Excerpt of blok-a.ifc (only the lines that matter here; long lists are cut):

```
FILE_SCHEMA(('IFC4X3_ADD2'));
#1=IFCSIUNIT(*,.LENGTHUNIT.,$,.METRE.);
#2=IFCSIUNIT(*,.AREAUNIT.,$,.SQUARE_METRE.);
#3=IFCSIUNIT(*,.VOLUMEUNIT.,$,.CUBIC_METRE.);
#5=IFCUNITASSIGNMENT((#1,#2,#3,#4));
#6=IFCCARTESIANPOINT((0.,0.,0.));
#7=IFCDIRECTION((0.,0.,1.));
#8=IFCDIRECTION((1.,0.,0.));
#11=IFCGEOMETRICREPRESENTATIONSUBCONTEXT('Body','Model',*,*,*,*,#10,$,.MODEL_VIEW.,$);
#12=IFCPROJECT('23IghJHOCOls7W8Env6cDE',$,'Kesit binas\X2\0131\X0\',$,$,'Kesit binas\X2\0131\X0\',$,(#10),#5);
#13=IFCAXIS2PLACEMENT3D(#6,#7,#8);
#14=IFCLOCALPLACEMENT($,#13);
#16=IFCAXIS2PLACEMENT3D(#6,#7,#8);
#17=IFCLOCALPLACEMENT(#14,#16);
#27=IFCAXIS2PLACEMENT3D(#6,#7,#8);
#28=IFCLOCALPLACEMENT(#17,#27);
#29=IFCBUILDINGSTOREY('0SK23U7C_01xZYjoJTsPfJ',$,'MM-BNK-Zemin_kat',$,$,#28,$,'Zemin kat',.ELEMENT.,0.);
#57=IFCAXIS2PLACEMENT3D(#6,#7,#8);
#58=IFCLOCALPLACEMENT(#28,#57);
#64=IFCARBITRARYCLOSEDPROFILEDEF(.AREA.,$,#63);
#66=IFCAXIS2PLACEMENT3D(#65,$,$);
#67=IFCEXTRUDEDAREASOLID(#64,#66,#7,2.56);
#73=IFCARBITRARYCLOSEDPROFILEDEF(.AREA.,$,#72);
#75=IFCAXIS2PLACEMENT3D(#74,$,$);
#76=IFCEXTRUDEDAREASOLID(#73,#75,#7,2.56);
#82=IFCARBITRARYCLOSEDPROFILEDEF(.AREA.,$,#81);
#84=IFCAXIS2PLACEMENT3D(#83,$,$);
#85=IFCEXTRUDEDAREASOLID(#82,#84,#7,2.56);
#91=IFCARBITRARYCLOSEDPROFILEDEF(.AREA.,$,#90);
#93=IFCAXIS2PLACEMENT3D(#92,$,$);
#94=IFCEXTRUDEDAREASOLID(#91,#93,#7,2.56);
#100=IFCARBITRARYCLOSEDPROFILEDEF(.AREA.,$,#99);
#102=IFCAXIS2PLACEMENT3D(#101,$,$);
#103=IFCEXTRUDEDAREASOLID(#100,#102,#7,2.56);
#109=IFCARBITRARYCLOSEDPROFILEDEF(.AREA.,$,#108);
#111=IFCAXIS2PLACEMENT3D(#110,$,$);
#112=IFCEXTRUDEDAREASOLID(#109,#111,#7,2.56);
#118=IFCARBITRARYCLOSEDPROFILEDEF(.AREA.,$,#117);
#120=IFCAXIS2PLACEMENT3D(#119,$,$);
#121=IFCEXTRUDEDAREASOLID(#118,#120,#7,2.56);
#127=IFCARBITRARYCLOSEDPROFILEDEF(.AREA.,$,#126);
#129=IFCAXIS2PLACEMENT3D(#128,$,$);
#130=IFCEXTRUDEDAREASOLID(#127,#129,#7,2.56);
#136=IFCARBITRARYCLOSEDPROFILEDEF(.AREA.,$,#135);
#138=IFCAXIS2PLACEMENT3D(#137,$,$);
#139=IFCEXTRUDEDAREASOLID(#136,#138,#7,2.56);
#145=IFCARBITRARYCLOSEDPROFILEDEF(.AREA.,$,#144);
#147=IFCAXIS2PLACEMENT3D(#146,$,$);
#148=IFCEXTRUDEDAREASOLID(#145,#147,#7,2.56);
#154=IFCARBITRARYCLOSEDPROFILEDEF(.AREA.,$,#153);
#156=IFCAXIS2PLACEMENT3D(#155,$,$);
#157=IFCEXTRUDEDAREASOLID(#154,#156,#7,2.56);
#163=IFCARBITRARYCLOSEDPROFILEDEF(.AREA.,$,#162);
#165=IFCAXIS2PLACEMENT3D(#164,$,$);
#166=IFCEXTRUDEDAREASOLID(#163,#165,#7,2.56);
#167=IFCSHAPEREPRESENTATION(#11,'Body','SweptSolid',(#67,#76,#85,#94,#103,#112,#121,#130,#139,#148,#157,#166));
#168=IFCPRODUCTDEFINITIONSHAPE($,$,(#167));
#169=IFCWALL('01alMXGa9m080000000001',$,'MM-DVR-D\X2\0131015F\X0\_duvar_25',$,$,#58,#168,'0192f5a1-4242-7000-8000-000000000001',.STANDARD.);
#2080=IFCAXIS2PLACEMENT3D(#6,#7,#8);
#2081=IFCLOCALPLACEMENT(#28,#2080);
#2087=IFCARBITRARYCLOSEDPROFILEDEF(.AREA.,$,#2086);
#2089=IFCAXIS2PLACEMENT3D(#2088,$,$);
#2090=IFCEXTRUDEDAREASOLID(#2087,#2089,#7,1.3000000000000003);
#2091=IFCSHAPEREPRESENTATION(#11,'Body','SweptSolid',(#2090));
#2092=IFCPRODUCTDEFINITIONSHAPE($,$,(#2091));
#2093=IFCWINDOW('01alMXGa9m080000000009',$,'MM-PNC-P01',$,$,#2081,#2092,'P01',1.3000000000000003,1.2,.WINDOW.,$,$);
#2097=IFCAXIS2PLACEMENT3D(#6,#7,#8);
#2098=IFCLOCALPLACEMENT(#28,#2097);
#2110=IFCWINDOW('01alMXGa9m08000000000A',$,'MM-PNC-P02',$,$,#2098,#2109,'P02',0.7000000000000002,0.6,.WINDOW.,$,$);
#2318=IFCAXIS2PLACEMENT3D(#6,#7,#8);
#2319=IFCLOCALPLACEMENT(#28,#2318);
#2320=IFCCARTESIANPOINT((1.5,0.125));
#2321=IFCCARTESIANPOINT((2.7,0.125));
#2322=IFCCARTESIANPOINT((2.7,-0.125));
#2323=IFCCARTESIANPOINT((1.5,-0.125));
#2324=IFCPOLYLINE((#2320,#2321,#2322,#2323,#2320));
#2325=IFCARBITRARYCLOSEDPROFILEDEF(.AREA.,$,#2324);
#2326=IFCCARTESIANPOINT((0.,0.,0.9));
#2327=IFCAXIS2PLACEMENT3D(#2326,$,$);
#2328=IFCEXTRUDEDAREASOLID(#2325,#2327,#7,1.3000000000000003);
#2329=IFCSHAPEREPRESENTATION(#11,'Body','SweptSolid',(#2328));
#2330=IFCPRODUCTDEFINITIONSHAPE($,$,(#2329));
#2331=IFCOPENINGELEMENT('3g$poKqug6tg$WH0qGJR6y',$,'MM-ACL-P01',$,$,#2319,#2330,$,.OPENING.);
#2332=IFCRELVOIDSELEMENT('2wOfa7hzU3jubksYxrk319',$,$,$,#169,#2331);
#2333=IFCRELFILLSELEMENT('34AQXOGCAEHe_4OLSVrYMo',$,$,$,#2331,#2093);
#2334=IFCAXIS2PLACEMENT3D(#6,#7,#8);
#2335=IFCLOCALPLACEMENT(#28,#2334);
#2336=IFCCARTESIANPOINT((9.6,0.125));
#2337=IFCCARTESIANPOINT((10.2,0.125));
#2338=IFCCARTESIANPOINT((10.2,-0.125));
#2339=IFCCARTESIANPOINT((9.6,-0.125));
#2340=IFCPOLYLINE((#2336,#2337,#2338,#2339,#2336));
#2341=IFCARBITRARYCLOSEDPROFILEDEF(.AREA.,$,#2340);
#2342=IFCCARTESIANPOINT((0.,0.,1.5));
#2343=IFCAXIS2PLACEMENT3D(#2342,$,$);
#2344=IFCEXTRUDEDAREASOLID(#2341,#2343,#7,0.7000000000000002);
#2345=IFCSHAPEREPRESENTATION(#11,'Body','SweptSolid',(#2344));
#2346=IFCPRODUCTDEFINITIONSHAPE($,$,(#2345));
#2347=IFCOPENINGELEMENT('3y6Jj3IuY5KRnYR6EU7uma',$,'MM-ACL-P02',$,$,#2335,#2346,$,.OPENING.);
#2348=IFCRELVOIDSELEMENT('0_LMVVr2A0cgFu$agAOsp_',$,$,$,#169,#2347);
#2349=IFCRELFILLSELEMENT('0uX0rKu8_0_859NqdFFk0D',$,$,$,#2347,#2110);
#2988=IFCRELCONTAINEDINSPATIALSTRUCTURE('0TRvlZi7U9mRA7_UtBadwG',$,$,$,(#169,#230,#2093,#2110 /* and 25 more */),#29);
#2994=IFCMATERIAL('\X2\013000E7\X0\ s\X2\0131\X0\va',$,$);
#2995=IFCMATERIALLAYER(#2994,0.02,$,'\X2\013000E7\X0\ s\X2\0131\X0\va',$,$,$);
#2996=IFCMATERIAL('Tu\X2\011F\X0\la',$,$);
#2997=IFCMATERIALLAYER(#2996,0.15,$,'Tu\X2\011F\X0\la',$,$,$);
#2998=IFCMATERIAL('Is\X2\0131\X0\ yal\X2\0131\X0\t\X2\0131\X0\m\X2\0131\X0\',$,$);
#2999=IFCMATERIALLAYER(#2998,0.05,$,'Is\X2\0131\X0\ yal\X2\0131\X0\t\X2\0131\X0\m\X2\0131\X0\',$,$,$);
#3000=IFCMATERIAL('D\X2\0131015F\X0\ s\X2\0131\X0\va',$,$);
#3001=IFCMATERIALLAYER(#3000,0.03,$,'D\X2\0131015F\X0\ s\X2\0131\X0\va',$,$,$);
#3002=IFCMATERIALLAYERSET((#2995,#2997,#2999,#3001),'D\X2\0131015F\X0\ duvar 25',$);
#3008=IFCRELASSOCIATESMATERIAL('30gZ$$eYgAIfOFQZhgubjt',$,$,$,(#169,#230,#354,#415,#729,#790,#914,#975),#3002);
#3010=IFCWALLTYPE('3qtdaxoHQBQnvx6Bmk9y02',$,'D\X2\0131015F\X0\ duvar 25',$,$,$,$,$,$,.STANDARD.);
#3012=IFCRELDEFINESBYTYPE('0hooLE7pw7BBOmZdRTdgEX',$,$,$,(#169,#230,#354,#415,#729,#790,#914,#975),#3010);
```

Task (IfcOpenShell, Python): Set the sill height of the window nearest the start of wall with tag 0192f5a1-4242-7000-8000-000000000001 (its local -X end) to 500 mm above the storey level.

```python
import numpy as np
import ifcopenshell
import ifcopenshell.api.geometry
import ifcopenshell.geom
import ifcopenshell.util.element
import ifcopenshell.util.placement
import ifcopenshell.util.shape
import ifcopenshell.util.unit

model = ifcopenshell.open("blok-a.ifc")
unit_scale = ifcopenshell.util.unit.calculate_unit_scale(model)

window = model.by_guid("01alMXGa9m080000000009")
opening = window.FillsVoids[0].RelatingOpeningElement
storey = ifcopenshell.util.element.get_container(window, ifc_class="IfcBuildingStorey")
level = ifcopenshell.util.placement.get_local_placement(storey.ObjectPlacement)[2, 3]

# The opening's origin need not be at the sill, so measure its lowest point.
shape = ifcopenshell.geom.create_shape(ifcopenshell.geom.settings(), opening)
bottom = ifcopenshell.util.shape.get_shape_bottom_elevation(shape, shape.geometry) / unit_scale
dz = level + 0.5 / unit_scale - bottom

shift = np.array([0.0, 0.0, dz])
# The window is not placed relative to its opening, so move both.
for product in (opening, window):
    matrix = ifcopenshell.util.placement.get_local_placement(product.ObjectPlacement)
    matrix[:3, 3] += shift
    ifcopenshell.api.geometry.edit_object_placement(model, product=product, matrix=matrix, is_si=False)

print(f"moved by {dz * unit_scale:+.3f} m")

model.write("blok-a-out.ifc")
```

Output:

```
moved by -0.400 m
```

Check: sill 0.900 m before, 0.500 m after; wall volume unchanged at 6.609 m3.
